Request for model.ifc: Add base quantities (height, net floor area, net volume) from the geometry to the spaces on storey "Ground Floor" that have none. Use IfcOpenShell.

First a look at what the model holds.

```python
import ifcopenshell
import ifcopenshell.util.element
import ifcopenshell.util.unit

model = ifcopenshell.open("model.ifc")
print(model.schema)
for unit_type in ("LENGTHUNIT", "AREAUNIT", "VOLUMEUNIT"):
    print(unit_type, ifcopenshell.util.unit.calculate_unit_scale(model, unit_type))
storey = next(s for s in model.by_type("IfcBuildingStorey") if s.Name == "Ground Floor")
spaces = [e for e in ifcopenshell.util.element.get_decomposition(storey) if e.is_a("IfcSpace")]
for e in sorted(spaces, key=lambda e: e.id()):
    print(e.id(), e.is_a(), e.Name, list(ifcopenshell.util.element.get_psets(e, qtos_only=True)), sep=" | ")
```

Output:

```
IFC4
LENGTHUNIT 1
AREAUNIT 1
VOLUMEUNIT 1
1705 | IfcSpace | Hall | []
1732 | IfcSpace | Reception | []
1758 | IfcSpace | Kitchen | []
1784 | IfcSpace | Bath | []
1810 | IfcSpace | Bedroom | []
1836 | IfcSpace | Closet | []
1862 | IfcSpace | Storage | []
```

```python
import ifcopenshell
import ifcopenshell.api.pset
import ifcopenshell.geom
import ifcopenshell.util.element
import ifcopenshell.util.shape
import ifcopenshell.util.unit

model = ifcopenshell.open("model.ifc")
unit_scale = ifcopenshell.util.unit.calculate_unit_scale(model)
area_scale = ifcopenshell.util.unit.calculate_unit_scale(model, "AREAUNIT")
volume_scale = ifcopenshell.util.unit.calculate_unit_scale(model, "VOLUMEUNIT")
settings = ifcopenshell.geom.settings()

storey = next(s for s in model.by_type("IfcBuildingStorey") if s.Name == "Ground Floor")
spaces = [e for e in ifcopenshell.util.element.get_decomposition(storey) if e.is_a("IfcSpace")]

for e in sorted(spaces, key=lambda e: e.id()):
    if ifcopenshell.util.element.get_psets(e, qtos_only=True, should_inherit=False):
        continue
    # Geometry comes back in metres, in the element's own axes.
    shape = ifcopenshell.geom.create_shape(settings, e)
    values = {
        "Height": ifcopenshell.util.shape.get_z(shape.geometry) / unit_scale,
        "NetFloorArea": ifcopenshell.util.shape.get_footprint_area(shape.geometry) / area_scale,
        "NetVolume": ifcopenshell.util.shape.get_volume(shape.geometry) / volume_scale,
    }
    qto = ifcopenshell.api.pset.add_qto(model, product=e, name="Qto_SpaceBaseQuantities")
    ifcopenshell.api.pset.edit_qto(model, qto=qto, properties=values)
    print(e.id(), {k: round(v, 3) for k, v in values.items()})

model.write("model_updated.ifc")
```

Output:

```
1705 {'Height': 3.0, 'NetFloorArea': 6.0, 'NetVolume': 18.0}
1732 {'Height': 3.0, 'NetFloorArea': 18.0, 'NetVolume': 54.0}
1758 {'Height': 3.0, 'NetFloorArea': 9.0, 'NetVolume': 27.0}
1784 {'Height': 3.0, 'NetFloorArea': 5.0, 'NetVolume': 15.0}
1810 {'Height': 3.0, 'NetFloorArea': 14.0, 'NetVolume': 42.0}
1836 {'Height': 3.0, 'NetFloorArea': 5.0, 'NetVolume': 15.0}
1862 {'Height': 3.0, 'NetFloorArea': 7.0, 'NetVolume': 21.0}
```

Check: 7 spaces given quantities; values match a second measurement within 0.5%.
